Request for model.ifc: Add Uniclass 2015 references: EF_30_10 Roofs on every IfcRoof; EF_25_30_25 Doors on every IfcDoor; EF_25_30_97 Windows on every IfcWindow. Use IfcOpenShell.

First a look at what the model holds.

```python
import ifcopenshell

model = ifcopenshell.open("model.ifc")
print(model.schema)
print("classifications:", [c.Name for c in model.by_type("IfcClassification")])
for ifc_class in ("IfcDoor", "IfcRoof", "IfcStair", "IfcWall", "IfcWindow"):
    print(ifc_class, len(model.by_type(ifc_class)))
```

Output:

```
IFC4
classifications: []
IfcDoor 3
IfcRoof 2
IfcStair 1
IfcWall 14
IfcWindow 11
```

```python
import ifcopenshell
import ifcopenshell.api.classification

model = ifcopenshell.open("model.ifc")

system = ifcopenshell.api.classification.add_classification(model, classification="Uniclass 2015")

codes = {
    "IfcRoof": ("EF_30_10", "Roofs"),
    "IfcDoor": ("EF_25_30_25", "Doors"),
    "IfcWindow": ("EF_25_30_97", "Windows"),
}
for ifc_class, (code, name) in codes.items():
    products = model.by_type(ifc_class)
    ifcopenshell.api.classification.add_reference(
        model, products=products, classification=system, identification=code, name=name
    )
    print(code, len(products))

model.write("model_updated.ifc")
```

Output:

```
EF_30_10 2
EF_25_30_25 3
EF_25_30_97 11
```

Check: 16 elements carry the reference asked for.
